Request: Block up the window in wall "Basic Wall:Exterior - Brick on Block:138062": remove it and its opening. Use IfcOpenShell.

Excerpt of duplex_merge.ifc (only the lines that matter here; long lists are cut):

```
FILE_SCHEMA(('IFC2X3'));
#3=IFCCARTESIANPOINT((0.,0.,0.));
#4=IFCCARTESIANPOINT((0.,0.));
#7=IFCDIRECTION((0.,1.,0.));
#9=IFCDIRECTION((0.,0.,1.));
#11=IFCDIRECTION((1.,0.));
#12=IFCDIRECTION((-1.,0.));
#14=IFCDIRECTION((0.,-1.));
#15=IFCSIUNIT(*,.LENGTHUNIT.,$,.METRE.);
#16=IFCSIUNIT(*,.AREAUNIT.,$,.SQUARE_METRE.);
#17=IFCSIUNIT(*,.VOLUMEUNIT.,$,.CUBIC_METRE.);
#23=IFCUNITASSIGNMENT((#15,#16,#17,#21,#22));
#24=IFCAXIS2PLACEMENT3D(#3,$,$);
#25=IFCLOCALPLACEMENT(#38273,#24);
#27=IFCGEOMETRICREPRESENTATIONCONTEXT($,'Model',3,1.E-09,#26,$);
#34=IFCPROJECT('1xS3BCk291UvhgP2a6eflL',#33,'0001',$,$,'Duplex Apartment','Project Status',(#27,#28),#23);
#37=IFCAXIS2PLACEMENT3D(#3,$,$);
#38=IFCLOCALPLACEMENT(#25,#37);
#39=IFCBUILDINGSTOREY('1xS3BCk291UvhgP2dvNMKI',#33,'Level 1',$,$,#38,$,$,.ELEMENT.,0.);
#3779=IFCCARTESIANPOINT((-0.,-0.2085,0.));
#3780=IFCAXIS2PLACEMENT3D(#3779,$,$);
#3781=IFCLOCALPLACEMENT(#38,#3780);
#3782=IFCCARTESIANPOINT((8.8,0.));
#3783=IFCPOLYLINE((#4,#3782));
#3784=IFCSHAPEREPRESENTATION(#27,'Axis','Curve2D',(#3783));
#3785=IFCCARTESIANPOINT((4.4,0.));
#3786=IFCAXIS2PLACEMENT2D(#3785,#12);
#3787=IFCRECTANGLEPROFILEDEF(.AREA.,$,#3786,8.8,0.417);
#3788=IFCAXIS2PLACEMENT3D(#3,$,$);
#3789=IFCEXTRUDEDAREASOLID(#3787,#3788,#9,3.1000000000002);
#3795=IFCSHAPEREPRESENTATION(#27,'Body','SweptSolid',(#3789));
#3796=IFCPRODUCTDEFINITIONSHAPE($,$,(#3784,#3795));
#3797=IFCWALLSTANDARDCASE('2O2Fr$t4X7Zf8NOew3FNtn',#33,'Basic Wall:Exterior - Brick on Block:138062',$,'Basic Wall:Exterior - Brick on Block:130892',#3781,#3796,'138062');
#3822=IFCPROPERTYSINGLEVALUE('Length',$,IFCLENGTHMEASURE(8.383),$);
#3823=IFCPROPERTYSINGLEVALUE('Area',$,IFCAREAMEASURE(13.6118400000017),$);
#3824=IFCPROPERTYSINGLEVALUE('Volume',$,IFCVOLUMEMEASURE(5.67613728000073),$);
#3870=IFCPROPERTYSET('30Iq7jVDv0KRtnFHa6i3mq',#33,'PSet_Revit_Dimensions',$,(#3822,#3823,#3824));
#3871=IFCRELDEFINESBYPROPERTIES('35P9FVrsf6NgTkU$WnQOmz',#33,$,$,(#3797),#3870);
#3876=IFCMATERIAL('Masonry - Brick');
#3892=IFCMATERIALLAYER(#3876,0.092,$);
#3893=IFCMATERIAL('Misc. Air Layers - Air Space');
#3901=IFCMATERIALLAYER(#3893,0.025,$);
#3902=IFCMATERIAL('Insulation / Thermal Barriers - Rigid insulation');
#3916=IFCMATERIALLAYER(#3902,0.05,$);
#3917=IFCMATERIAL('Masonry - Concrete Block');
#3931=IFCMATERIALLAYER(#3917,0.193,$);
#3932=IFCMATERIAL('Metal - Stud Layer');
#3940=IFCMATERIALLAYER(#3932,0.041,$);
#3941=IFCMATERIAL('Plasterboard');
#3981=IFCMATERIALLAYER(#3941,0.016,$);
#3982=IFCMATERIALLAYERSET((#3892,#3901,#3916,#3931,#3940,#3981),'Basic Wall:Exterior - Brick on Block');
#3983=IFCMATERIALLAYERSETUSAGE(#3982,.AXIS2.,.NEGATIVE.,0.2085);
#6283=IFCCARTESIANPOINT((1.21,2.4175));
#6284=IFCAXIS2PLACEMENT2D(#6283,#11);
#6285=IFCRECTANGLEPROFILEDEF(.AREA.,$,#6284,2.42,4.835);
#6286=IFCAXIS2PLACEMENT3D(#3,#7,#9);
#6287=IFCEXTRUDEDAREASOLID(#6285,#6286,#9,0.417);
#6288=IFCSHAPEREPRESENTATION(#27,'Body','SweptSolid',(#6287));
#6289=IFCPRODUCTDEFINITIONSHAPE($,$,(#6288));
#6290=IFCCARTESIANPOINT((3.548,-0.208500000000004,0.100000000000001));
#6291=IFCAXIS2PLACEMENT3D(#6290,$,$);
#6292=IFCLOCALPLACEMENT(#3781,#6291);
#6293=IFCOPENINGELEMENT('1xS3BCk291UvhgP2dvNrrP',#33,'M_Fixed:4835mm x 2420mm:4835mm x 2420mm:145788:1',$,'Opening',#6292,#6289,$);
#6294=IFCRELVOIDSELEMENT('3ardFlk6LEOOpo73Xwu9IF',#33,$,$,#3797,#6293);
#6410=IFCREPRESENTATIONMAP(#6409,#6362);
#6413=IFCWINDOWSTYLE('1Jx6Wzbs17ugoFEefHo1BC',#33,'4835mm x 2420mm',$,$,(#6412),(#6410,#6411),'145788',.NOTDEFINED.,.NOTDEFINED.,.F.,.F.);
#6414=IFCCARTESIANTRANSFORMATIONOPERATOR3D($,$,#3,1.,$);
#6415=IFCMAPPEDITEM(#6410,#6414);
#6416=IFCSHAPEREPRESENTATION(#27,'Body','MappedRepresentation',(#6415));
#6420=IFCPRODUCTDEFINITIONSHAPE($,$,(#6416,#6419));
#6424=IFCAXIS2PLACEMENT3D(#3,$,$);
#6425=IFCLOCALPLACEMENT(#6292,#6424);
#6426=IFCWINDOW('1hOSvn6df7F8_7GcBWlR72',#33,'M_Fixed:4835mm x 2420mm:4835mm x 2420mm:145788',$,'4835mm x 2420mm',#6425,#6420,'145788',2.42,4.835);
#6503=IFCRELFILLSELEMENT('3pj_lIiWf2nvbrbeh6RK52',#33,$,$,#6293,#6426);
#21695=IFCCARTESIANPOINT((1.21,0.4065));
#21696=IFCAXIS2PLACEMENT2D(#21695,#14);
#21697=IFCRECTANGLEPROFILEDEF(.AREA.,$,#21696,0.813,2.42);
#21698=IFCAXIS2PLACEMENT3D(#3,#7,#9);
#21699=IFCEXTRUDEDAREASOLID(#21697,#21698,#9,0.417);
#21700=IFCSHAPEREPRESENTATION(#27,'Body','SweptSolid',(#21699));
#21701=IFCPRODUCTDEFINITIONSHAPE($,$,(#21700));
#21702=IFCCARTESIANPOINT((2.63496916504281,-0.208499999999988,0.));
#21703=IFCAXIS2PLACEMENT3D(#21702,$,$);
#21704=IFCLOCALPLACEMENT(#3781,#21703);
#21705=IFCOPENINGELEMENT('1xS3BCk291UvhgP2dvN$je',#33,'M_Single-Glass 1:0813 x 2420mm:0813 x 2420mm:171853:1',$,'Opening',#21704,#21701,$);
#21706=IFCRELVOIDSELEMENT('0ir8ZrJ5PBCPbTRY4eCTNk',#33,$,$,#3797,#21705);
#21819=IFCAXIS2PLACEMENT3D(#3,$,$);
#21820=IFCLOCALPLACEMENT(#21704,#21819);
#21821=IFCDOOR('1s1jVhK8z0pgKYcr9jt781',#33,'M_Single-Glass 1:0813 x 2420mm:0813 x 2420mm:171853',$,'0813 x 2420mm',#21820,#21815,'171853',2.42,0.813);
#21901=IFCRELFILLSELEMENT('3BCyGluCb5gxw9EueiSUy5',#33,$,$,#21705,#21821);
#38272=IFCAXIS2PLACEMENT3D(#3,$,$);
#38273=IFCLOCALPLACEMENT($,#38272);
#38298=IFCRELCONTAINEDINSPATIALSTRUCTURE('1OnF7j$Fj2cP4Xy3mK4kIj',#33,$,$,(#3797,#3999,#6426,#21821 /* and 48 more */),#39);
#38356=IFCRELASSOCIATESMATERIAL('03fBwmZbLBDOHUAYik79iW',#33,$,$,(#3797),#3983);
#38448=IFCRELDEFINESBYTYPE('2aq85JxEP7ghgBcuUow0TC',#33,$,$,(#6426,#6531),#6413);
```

```python
import ifcopenshell
import ifcopenshell.api.feature
import ifcopenshell.api.pset
import ifcopenshell.api.root
import ifcopenshell.geom
import ifcopenshell.util.element
import ifcopenshell.util.shape
import ifcopenshell.util.unit

model = ifcopenshell.open("duplex_merge.ifc")
area_scale = ifcopenshell.util.unit.calculate_unit_scale(model, "AREAUNIT")
volume_scale = ifcopenshell.util.unit.calculate_unit_scale(model, "VOLUMEUNIT")
settings = ifcopenshell.geom.settings()


def volume(element):
    """Net volume in cubic metres, openings subtracted."""
    shape = ifcopenshell.geom.create_shape(settings, element)
    return ifcopenshell.util.shape.get_volume(shape.geometry)


window = model.by_id(6426)
opening = window.FillsVoids[0].RelatingOpeningElement
wall = opening.VoidsElements[0].RelatingBuildingElement
before = volume(wall)

ifcopenshell.api.root.remove_product(model, product=window)
ifcopenshell.api.feature.remove_feature(model, feature=opening)

after = volume(wall)
thickness = 0.417  # wall thickness in metres

# Update the wall's stored quantities.
pset = model.by_id(ifcopenshell.util.element.get_pset(wall, "PSet_Revit_Dimensions", should_inherit=False)["id"])
ifcopenshell.api.pset.edit_pset(model, pset=pset, properties={
    "Area": model.create_entity("IfcAreaMeasure", after / thickness / area_scale),
    "Volume": model.create_entity("IfcVolumeMeasure", after / volume_scale),
})

print(f"wall volume {before:.3f} -> {after:.3f} m3")

model.write("duplex_merge_edited.ifc")
```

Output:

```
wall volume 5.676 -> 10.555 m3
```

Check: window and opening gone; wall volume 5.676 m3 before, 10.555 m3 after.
